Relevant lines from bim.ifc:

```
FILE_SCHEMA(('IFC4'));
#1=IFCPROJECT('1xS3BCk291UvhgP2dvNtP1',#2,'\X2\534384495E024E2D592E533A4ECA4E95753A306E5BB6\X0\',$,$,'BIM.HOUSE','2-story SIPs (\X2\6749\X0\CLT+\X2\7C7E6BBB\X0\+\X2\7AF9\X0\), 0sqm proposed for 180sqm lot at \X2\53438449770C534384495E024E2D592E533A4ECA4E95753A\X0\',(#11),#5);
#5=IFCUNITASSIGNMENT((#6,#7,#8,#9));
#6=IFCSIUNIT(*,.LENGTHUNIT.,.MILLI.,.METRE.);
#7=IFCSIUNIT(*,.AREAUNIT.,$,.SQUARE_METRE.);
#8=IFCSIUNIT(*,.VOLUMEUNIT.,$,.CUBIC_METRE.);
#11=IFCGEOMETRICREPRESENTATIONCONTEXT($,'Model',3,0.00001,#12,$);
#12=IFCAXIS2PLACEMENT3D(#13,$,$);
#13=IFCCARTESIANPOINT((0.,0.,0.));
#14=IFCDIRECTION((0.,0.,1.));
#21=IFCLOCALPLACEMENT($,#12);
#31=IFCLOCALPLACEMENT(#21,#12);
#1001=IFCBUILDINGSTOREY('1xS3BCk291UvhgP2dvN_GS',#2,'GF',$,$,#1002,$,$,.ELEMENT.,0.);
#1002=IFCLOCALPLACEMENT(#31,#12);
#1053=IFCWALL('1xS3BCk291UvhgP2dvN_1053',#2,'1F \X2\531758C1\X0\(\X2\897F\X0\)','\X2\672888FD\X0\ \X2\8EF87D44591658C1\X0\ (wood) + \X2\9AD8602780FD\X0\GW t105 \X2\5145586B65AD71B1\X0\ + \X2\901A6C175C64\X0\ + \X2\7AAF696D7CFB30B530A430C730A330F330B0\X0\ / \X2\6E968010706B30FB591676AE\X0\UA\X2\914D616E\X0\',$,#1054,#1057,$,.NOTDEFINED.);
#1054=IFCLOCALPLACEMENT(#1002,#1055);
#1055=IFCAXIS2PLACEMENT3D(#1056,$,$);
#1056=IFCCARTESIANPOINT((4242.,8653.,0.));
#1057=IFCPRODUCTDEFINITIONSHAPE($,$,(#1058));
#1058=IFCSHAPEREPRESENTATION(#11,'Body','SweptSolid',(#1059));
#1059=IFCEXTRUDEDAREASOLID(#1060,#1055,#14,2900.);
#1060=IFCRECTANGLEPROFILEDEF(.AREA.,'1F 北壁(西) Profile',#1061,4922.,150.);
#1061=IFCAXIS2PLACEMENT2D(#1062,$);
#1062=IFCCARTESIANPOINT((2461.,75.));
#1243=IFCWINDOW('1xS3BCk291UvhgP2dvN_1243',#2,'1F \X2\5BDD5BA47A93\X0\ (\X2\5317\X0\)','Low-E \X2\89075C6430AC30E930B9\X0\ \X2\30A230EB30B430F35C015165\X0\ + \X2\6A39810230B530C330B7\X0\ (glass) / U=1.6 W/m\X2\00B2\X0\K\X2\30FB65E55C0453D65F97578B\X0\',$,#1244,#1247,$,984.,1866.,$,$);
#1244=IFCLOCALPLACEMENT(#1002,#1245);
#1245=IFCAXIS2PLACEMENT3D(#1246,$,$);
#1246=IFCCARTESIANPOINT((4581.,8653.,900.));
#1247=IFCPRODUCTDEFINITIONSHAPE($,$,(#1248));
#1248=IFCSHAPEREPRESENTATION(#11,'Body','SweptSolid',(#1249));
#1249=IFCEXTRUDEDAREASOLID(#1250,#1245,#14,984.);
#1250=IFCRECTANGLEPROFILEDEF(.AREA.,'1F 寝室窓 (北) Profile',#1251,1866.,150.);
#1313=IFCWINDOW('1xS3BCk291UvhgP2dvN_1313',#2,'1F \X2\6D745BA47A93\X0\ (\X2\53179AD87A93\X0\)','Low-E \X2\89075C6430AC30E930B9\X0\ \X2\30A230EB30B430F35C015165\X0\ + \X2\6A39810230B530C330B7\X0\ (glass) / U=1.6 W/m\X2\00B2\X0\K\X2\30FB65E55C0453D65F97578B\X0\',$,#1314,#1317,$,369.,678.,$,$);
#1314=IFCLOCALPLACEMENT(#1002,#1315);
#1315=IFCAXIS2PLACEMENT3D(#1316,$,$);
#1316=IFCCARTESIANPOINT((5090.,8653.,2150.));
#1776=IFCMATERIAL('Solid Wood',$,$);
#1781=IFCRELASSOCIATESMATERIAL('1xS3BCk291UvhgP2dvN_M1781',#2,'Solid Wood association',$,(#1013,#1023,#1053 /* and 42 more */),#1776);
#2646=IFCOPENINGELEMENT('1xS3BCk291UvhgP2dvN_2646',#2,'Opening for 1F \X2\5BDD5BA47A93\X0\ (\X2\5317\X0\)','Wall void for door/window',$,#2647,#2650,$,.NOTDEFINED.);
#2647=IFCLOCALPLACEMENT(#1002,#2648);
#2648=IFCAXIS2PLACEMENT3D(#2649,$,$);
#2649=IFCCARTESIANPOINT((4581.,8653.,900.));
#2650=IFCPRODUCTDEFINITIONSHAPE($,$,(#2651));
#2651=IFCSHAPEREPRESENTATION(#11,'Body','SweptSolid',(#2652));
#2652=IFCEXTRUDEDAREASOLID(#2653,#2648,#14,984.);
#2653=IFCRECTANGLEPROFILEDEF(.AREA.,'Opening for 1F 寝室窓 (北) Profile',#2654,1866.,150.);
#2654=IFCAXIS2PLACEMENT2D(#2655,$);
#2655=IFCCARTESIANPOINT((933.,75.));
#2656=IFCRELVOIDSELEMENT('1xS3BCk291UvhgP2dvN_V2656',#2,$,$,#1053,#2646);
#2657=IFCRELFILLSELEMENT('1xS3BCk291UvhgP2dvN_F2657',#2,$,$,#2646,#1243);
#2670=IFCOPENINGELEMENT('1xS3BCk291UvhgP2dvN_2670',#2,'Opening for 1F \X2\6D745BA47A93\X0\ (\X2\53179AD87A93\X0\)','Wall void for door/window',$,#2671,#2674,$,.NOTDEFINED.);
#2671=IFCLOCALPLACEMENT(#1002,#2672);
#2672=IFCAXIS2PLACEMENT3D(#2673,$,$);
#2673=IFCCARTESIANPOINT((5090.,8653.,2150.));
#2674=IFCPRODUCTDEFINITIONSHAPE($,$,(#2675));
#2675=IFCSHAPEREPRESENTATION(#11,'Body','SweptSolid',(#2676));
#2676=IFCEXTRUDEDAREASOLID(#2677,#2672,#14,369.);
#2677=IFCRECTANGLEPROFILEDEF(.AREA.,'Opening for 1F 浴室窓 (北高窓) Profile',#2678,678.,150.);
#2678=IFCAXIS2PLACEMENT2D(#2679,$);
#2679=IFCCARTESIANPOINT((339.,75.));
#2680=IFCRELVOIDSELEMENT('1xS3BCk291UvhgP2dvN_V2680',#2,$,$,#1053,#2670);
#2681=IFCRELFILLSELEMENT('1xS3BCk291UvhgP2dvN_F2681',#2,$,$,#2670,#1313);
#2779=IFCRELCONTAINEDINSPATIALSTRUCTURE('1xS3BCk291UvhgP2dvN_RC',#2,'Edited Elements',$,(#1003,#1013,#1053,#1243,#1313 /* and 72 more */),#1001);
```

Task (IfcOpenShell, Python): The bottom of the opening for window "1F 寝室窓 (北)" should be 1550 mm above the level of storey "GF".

```python
import numpy as np
import ifcopenshell
import ifcopenshell.api.geometry
import ifcopenshell.geom
import ifcopenshell.util.element
import ifcopenshell.util.placement
import ifcopenshell.util.shape
import ifcopenshell.util.unit

model = ifcopenshell.open("bim.ifc")
unit_scale = ifcopenshell.util.unit.calculate_unit_scale(model)

window = model.by_guid("1xS3BCk291UvhgP2dvN_1243")
opening = window.FillsVoids[0].RelatingOpeningElement
storey = ifcopenshell.util.element.get_container(window, ifc_class="IfcBuildingStorey")
level = ifcopenshell.util.placement.get_local_placement(storey.ObjectPlacement)[2, 3]

# The opening's origin need not be at the sill, so measure its lowest point.
shape = ifcopenshell.geom.create_shape(ifcopenshell.geom.settings(), opening)
bottom = ifcopenshell.util.shape.get_shape_bottom_elevation(shape, shape.geometry) / unit_scale
dz = level + 1.55 / unit_scale - bottom

shift = np.array([0.0, 0.0, dz])
# The window is not placed relative to its opening, so move both.
for product in (opening, window):
    matrix = ifcopenshell.util.placement.get_local_placement(product.ObjectPlacement)
    matrix[:3, 3] += shift
    ifcopenshell.api.geometry.edit_object_placement(model, product=product, matrix=matrix, is_si=False)

print(f"moved by {dz * unit_scale:+.3f} m")

model.write("bim_v2.ifc")
```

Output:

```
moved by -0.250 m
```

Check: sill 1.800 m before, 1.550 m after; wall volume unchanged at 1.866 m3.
